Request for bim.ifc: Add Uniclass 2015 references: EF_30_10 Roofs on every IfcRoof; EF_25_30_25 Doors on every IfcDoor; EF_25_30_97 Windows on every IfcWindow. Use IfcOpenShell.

First a look at what the model holds.

```python
import ifcopenshell

model = ifcopenshell.open("bim.ifc")
print(model.schema)
print("classifications:", [c.Name for c in model.by_type("IfcClassification")])
for ifc_class in ("IfcDoor", "IfcRoof", "IfcStair", "IfcWall", "IfcWindow"):
    print(ifc_class, len(model.by_type(ifc_class)))
```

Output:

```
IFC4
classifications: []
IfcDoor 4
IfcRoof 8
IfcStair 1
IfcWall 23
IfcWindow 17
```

```python
import ifcopenshell
import ifcopenshell.api.classification

model = ifcopenshell.open("bim.ifc")

system = ifcopenshell.api.classification.add_classification(model, classification="Uniclass 2015")

codes = {
    "IfcRoof": ("EF_30_10", "Roofs"),
    "IfcDoor": ("EF_25_30_25", "Doors"),
    "IfcWindow": ("EF_25_30_97", "Windows"),
}
for ifc_class, (code, name) in codes.items():
    products = model.by_type(ifc_class)
    ifcopenshell.api.classification.add_reference(
        model, products=products, classification=system, identification=code, name=name
    )
    print(code, len(products))

model.write("bim_edited.ifc")
```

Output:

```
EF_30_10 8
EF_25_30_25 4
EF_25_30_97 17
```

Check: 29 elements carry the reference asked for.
